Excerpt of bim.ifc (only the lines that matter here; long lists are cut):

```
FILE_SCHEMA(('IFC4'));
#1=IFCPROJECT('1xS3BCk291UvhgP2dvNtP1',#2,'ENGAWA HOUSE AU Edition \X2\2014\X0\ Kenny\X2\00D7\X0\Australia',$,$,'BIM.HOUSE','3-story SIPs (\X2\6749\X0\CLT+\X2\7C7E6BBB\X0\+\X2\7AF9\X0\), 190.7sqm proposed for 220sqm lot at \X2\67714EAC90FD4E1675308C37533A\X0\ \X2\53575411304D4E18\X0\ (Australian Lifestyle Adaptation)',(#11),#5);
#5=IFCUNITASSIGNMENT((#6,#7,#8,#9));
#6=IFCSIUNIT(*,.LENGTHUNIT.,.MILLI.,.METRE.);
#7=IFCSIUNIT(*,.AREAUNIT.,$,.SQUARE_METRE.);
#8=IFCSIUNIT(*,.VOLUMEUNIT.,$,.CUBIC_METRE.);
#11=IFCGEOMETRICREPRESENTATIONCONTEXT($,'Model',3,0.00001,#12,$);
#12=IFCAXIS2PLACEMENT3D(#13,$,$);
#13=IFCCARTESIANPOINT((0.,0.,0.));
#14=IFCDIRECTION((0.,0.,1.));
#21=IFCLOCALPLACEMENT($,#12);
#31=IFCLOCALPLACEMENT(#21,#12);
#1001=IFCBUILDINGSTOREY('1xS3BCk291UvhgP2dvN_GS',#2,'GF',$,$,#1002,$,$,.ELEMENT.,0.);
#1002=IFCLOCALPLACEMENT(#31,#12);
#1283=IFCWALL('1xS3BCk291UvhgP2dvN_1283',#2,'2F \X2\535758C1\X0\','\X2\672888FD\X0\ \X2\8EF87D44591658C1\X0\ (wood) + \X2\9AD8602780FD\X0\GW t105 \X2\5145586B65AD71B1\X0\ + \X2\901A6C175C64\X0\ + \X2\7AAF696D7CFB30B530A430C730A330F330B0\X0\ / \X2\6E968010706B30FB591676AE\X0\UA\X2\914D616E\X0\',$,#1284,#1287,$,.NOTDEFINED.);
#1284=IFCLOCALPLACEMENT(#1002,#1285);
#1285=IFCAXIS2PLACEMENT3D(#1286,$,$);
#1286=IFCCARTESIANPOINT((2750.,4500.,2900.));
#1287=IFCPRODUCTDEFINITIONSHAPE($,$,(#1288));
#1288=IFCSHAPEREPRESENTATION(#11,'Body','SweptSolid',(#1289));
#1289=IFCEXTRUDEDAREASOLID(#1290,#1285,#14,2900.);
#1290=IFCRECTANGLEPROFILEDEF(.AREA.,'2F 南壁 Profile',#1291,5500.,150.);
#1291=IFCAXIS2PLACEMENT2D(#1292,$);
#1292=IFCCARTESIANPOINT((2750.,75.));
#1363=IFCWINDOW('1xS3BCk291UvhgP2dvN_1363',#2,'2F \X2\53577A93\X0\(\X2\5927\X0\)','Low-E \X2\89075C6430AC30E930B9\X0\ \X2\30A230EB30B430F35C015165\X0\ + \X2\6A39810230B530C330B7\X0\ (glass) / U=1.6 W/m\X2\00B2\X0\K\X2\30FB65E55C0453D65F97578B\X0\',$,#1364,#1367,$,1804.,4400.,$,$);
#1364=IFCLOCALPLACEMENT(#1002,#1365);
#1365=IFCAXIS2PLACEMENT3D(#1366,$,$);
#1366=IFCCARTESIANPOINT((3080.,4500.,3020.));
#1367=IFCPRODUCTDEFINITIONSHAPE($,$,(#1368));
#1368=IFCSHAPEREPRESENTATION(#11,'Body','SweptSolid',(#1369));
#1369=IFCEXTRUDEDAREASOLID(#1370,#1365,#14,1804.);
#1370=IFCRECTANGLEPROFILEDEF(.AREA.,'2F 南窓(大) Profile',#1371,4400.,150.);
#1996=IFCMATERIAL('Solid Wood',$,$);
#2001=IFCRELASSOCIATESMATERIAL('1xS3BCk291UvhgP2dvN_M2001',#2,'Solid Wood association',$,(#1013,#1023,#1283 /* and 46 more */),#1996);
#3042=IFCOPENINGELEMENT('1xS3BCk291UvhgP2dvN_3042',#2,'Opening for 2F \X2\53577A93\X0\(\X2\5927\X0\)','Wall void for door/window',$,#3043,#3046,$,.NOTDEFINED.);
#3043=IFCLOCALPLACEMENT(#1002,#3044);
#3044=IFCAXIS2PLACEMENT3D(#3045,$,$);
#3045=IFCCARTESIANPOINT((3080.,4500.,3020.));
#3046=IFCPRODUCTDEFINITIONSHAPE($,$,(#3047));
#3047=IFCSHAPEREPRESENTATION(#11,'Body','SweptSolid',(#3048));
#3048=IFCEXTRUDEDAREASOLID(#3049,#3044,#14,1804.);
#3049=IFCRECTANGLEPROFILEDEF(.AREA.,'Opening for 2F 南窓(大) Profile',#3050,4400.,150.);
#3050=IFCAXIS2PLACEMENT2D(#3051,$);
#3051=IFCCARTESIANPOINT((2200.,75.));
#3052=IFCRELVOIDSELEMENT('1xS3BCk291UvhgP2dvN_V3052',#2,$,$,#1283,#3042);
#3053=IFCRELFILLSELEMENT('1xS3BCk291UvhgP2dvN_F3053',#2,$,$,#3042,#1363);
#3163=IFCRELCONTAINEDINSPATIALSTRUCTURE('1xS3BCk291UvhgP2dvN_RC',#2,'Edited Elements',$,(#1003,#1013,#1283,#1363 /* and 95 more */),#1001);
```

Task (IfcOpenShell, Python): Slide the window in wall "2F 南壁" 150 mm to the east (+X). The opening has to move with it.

```python
import ifcopenshell
import ifcopenshell.api.geometry
import ifcopenshell.util.placement

model = ifcopenshell.open("bim.ifc")

window = model.by_guid("1xS3BCk291UvhgP2dvN_1363")
opening = window.FillsVoids[0].RelatingOpeningElement
wall = opening.VoidsElements[0].RelatingBuildingElement

wall_matrix = ifcopenshell.util.placement.get_local_placement(wall.ObjectPlacement)
shift = wall_matrix[:3, 0] * 150.0
before = ifcopenshell.util.placement.get_local_placement(window.ObjectPlacement)[:3, 3].copy()

# The window is not placed relative to its opening, so move both.
for product in (opening, window):
    matrix = ifcopenshell.util.placement.get_local_placement(product.ObjectPlacement)
    matrix[:3, 3] += shift
    ifcopenshell.api.geometry.edit_object_placement(model, product=product, matrix=matrix, is_si=False)

after = ifcopenshell.util.placement.get_local_placement(window.ObjectPlacement)[:3, 3]
print("window moved by", (after - before).round(3) + 0.0)

model.write("bim-out.ifc")
```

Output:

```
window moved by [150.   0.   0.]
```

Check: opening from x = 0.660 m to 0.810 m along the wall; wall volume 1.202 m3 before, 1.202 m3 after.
